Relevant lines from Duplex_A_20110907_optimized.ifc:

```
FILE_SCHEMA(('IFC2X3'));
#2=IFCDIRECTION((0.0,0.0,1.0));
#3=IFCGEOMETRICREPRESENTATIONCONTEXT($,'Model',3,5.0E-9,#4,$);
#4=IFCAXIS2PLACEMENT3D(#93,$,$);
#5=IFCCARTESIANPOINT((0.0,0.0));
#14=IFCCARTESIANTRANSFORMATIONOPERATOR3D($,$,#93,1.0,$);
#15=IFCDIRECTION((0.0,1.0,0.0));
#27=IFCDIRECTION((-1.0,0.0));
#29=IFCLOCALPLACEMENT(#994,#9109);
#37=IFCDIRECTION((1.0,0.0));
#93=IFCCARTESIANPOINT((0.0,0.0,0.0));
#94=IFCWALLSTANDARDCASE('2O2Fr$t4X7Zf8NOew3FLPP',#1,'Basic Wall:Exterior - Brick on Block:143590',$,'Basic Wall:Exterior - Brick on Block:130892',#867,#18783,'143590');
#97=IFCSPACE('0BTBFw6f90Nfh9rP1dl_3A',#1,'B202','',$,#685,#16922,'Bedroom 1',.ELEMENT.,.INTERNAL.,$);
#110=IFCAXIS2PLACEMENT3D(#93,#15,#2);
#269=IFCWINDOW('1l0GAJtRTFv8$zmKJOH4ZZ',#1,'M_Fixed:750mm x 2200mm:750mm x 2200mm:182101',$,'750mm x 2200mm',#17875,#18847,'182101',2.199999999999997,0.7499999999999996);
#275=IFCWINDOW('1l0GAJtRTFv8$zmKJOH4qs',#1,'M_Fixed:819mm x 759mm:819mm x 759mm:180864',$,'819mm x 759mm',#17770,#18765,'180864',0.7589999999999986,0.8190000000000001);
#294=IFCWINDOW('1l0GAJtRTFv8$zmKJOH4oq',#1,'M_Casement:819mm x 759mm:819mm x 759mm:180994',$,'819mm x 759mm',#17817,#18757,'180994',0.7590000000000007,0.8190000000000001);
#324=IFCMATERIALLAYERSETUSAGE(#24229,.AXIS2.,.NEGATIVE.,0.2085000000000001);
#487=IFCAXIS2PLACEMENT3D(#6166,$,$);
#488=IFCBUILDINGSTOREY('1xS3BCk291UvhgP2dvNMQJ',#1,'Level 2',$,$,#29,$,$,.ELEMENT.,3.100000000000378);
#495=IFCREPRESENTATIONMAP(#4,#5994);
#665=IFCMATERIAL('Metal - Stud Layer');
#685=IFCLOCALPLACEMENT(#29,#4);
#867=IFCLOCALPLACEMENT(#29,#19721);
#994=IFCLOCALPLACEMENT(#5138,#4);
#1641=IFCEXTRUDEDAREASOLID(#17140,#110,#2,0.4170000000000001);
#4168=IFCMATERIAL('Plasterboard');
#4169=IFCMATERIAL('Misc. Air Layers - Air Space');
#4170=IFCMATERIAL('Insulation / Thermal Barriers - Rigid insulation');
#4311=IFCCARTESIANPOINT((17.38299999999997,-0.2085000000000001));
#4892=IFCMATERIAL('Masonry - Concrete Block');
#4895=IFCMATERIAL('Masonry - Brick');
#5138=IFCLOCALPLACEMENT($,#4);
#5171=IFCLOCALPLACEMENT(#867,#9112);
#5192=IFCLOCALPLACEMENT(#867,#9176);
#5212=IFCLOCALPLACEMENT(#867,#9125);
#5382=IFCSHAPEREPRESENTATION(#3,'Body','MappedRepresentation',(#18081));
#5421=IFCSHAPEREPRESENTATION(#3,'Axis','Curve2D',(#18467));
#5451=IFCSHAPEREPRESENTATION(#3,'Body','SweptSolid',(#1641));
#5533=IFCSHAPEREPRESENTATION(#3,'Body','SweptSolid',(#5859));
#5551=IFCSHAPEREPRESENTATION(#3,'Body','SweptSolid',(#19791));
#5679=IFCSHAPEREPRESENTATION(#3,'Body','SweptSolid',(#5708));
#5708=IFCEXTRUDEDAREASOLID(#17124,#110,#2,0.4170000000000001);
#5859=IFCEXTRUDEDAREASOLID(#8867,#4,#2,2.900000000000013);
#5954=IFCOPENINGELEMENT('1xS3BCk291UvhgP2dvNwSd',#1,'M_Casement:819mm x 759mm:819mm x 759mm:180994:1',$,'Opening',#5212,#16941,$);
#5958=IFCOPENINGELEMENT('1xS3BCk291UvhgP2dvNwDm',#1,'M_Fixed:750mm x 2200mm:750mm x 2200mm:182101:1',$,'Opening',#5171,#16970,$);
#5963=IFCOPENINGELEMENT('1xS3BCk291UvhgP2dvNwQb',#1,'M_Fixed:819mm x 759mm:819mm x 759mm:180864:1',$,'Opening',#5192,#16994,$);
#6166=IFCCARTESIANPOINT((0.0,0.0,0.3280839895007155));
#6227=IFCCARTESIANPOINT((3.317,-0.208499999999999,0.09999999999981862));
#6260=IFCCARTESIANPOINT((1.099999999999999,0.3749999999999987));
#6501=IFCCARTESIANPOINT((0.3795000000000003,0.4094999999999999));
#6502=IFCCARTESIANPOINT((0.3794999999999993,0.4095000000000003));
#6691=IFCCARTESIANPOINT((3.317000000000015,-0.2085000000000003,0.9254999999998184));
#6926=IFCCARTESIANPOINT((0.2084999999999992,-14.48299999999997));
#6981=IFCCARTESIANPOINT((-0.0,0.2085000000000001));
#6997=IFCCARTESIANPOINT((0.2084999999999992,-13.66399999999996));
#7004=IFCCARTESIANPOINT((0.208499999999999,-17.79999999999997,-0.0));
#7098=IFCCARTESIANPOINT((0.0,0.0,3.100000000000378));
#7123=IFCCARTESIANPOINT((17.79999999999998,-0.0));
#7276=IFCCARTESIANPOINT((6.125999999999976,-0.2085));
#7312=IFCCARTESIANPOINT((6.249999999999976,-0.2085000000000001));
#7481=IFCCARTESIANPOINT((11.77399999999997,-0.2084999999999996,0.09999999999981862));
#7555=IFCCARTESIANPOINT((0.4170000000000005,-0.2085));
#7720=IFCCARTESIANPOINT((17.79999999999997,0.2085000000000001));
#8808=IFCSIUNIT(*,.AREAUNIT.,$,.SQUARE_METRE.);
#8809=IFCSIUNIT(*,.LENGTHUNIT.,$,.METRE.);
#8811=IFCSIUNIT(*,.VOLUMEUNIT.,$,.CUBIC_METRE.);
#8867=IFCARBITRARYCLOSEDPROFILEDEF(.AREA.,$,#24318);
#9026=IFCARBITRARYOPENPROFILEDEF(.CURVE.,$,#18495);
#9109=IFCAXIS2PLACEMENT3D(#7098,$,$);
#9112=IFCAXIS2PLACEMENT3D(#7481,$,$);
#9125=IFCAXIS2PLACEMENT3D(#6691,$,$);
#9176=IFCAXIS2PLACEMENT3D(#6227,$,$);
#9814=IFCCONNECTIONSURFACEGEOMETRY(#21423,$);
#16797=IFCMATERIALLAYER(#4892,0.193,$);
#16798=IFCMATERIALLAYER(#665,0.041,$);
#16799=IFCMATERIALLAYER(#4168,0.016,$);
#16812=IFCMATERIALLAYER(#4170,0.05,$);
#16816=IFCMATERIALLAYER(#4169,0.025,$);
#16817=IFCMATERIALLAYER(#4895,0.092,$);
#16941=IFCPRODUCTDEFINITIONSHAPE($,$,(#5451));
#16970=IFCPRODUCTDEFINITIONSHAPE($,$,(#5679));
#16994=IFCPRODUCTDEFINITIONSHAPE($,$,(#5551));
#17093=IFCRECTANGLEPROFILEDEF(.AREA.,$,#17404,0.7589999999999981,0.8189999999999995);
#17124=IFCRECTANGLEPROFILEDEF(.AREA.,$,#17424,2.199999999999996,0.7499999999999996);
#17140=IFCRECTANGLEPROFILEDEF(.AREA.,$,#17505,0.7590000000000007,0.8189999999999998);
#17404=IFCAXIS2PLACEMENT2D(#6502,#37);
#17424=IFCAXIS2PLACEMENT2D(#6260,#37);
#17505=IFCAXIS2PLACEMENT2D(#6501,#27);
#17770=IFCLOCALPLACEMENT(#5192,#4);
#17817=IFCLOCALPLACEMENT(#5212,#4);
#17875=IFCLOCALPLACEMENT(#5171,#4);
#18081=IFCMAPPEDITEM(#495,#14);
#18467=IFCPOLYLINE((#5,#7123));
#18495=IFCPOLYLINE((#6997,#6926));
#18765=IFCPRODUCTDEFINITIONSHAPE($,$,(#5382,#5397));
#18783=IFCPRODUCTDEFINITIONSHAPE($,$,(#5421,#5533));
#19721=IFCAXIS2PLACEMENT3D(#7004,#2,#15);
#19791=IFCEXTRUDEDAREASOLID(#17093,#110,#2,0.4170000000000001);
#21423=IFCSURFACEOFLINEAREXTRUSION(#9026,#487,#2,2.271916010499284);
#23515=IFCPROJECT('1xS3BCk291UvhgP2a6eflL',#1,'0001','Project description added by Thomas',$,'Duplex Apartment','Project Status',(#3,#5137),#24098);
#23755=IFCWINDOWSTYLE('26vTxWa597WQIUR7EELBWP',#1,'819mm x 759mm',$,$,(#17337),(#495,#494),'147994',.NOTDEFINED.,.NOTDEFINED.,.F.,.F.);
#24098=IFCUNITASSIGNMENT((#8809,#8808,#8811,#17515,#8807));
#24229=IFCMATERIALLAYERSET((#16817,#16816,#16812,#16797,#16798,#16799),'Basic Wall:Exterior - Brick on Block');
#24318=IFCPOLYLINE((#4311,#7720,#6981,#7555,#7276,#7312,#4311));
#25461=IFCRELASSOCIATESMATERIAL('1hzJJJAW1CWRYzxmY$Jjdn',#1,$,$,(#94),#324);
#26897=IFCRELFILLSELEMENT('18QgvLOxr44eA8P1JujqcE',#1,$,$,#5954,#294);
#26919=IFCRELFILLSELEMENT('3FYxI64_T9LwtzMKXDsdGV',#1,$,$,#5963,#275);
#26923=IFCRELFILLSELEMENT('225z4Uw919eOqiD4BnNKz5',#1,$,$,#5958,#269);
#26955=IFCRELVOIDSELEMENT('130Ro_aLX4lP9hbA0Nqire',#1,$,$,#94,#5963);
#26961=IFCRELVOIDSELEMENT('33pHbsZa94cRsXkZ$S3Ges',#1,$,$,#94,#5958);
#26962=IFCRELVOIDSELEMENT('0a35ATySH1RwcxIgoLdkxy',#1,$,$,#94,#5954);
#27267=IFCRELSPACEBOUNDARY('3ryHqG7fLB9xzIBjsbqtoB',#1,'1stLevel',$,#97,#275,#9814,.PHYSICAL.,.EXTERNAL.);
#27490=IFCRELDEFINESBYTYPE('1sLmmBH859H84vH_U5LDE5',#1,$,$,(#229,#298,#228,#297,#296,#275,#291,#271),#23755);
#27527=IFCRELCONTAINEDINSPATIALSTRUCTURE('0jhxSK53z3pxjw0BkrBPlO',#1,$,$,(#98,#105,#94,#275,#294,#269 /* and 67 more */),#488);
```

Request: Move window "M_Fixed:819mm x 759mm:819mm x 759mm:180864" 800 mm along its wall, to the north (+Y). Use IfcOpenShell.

```python
import numpy as np
import ifcopenshell
import ifcopenshell.api.geometry
import ifcopenshell.util.placement
import ifcopenshell.util.unit

model = ifcopenshell.open("Duplex_A_20110907_optimized.ifc")
unit_scale = ifcopenshell.util.unit.calculate_unit_scale(model)

window = model.by_guid("1l0GAJtRTFv8$zmKJOH4qs")
opening = window.FillsVoids[0].RelatingOpeningElement
wall = opening.VoidsElements[0].RelatingBuildingElement

wall_matrix = ifcopenshell.util.placement.get_local_placement(wall.ObjectPlacement)
shift = wall_matrix[:3, 0] * 0.8 / unit_scale
before = ifcopenshell.util.placement.get_local_placement(window.ObjectPlacement)[:3, 3].copy()

# The window is placed relative to its opening, so it follows when the opening moves.
matrix = ifcopenshell.util.placement.get_local_placement(opening.ObjectPlacement)
matrix[:3, 3] += shift
ifcopenshell.api.geometry.edit_object_placement(
    model, product=opening, matrix=matrix, is_si=False, should_transform_children=True
)

# Space boundary surfaces are stored in each space's coordinates; move them too.
for rel in window.ProvidesBoundaries:
    if not rel.ConnectionGeometry:
        continue
    surface = rel.ConnectionGeometry.SurfaceOnRelatingElement
    space_matrix = ifcopenshell.util.placement.get_local_placement(rel.RelatingSpace.ObjectPlacement)
    point = np.array(surface.Position.Location.Coordinates) + space_matrix[:3, :3].T @ shift
    surface.Position = model.createIfcAxis2Placement3D(
        model.createIfcCartesianPoint(point.tolist()), surface.Position.Axis, surface.Position.RefDirection
    )

after = ifcopenshell.util.placement.get_local_placement(window.ObjectPlacement)[:3, 3]
print("window moved by", (after - before).round(3) + 0.0)

model.write("Duplex_A_20110907_optimized-out.ifc")
```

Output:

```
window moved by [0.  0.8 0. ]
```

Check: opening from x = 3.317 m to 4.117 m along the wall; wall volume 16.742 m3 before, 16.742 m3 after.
